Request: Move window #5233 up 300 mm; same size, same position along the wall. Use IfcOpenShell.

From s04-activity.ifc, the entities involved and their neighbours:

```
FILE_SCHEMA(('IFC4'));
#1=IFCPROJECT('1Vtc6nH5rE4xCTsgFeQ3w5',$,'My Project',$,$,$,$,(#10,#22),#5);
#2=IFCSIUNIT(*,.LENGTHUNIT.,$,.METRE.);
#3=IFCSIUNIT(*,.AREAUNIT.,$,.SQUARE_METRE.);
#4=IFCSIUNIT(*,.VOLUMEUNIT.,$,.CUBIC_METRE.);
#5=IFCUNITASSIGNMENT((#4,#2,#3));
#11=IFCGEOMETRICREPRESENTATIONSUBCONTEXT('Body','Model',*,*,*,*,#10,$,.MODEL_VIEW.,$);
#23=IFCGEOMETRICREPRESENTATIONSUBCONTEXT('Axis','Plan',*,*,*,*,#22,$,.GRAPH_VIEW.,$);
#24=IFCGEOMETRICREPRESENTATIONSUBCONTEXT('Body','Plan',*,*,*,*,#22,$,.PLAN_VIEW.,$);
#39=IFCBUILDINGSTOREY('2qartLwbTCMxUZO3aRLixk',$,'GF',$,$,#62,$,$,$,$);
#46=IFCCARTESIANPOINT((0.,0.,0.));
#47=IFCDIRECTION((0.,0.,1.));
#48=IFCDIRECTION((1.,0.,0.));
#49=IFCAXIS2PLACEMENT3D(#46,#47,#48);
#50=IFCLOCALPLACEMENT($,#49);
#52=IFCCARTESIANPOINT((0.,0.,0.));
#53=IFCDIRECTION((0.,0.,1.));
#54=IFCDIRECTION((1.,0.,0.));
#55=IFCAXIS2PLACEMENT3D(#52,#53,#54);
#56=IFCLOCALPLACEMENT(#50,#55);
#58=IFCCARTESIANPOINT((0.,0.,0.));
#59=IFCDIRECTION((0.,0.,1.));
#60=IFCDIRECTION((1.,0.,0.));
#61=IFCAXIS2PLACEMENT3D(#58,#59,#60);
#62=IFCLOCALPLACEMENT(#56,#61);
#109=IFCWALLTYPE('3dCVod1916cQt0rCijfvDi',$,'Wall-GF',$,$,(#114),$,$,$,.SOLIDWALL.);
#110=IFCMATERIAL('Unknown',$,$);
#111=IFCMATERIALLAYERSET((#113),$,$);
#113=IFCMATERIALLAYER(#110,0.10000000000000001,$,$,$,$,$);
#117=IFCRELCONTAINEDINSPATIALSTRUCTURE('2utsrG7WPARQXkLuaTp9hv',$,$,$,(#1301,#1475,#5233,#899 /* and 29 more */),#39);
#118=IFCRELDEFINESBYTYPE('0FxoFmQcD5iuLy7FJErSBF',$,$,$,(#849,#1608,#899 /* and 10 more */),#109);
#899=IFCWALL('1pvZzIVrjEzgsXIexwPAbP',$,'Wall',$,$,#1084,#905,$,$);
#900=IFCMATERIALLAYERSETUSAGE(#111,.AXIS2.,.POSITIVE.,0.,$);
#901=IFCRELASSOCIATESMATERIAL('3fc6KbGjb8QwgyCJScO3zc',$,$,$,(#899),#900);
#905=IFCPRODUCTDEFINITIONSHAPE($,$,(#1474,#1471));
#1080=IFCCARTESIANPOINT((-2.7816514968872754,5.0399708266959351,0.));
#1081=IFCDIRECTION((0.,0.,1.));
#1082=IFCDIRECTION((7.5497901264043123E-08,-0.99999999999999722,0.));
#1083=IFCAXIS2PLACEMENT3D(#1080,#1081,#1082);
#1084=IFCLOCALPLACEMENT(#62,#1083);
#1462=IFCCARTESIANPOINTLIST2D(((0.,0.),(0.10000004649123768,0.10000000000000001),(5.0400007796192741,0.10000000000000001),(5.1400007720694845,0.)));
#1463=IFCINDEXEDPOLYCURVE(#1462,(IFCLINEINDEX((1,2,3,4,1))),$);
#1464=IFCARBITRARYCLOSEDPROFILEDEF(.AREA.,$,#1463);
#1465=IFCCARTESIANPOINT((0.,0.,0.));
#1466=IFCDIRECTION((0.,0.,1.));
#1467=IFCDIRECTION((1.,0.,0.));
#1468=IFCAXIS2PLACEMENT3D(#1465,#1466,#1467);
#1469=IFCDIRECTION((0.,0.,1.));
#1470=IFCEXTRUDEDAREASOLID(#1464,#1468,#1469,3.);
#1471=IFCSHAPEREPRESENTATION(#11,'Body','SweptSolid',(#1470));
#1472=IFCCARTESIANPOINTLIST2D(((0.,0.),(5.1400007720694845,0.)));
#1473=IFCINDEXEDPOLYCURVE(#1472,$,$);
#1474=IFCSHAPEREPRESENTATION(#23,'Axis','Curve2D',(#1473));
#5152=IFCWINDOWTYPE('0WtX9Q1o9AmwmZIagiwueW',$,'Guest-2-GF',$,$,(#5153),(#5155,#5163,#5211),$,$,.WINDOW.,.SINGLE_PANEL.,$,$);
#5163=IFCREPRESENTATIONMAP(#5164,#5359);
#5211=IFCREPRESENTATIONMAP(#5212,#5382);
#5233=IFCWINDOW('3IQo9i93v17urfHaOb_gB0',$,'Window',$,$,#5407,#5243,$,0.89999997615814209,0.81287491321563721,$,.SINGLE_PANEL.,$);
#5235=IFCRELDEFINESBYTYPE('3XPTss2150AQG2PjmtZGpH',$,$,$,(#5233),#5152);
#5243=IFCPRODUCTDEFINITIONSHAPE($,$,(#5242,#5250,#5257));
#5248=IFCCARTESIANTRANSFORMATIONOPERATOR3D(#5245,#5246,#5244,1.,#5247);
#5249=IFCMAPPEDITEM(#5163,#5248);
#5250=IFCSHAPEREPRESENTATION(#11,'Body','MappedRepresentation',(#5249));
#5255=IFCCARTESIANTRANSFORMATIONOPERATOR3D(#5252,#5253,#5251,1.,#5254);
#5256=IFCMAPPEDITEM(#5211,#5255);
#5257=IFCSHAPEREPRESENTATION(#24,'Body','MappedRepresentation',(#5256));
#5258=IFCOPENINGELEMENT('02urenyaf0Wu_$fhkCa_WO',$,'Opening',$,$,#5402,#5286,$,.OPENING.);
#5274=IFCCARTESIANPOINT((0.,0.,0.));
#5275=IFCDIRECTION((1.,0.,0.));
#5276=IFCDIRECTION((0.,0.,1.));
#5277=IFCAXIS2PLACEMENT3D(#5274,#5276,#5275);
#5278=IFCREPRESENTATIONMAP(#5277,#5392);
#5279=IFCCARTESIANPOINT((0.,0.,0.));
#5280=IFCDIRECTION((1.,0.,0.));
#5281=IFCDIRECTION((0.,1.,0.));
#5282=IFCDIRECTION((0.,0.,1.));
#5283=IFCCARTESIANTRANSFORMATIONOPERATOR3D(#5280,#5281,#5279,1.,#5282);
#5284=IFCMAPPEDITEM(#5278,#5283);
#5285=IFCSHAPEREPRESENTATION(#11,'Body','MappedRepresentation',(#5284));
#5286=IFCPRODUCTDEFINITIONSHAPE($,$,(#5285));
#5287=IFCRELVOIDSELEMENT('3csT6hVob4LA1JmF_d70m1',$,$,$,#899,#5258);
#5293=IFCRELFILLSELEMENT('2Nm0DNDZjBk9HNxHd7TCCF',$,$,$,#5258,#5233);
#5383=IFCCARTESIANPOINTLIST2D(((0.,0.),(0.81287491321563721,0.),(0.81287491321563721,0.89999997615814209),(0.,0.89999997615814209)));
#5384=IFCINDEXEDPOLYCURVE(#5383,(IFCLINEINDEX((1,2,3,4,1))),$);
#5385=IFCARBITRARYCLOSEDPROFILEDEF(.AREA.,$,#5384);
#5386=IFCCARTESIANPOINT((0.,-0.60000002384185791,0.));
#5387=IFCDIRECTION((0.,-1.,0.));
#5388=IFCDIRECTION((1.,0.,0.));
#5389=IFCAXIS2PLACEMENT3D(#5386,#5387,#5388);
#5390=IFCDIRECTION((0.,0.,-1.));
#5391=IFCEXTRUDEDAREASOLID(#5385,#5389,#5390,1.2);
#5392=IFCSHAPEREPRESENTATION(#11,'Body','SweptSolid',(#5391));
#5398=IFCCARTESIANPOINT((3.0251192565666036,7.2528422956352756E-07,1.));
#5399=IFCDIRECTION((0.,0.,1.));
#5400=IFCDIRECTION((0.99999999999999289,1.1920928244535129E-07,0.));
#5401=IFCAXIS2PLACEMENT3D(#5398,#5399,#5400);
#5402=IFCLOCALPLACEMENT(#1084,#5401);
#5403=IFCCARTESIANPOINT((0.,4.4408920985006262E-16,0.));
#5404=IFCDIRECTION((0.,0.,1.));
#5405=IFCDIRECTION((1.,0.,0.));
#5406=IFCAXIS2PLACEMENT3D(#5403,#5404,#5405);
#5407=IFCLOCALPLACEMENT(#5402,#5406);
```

```python
import numpy as np
import ifcopenshell
import ifcopenshell.api.geometry
import ifcopenshell.util.placement
import ifcopenshell.util.unit

model = ifcopenshell.open("s04-activity.ifc")
unit_scale = ifcopenshell.util.unit.calculate_unit_scale(model)

window = model.by_guid("3IQo9i93v17urfHaOb_gB0")
opening = window.FillsVoids[0].RelatingOpeningElement
dz = 0.3

shift = np.array([0.0, 0.0, dz])
# The window is placed relative to its opening, so it follows when the opening moves.
matrix = ifcopenshell.util.placement.get_local_placement(opening.ObjectPlacement)
matrix[:3, 3] += shift
ifcopenshell.api.geometry.edit_object_placement(
    model, product=opening, matrix=matrix, is_si=False, should_transform_children=True
)

print(f"moved by {dz * unit_scale:+.3f} m")

model.write("s04-activity-out.ifc")
```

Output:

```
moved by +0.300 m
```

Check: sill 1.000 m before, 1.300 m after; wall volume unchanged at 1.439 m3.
